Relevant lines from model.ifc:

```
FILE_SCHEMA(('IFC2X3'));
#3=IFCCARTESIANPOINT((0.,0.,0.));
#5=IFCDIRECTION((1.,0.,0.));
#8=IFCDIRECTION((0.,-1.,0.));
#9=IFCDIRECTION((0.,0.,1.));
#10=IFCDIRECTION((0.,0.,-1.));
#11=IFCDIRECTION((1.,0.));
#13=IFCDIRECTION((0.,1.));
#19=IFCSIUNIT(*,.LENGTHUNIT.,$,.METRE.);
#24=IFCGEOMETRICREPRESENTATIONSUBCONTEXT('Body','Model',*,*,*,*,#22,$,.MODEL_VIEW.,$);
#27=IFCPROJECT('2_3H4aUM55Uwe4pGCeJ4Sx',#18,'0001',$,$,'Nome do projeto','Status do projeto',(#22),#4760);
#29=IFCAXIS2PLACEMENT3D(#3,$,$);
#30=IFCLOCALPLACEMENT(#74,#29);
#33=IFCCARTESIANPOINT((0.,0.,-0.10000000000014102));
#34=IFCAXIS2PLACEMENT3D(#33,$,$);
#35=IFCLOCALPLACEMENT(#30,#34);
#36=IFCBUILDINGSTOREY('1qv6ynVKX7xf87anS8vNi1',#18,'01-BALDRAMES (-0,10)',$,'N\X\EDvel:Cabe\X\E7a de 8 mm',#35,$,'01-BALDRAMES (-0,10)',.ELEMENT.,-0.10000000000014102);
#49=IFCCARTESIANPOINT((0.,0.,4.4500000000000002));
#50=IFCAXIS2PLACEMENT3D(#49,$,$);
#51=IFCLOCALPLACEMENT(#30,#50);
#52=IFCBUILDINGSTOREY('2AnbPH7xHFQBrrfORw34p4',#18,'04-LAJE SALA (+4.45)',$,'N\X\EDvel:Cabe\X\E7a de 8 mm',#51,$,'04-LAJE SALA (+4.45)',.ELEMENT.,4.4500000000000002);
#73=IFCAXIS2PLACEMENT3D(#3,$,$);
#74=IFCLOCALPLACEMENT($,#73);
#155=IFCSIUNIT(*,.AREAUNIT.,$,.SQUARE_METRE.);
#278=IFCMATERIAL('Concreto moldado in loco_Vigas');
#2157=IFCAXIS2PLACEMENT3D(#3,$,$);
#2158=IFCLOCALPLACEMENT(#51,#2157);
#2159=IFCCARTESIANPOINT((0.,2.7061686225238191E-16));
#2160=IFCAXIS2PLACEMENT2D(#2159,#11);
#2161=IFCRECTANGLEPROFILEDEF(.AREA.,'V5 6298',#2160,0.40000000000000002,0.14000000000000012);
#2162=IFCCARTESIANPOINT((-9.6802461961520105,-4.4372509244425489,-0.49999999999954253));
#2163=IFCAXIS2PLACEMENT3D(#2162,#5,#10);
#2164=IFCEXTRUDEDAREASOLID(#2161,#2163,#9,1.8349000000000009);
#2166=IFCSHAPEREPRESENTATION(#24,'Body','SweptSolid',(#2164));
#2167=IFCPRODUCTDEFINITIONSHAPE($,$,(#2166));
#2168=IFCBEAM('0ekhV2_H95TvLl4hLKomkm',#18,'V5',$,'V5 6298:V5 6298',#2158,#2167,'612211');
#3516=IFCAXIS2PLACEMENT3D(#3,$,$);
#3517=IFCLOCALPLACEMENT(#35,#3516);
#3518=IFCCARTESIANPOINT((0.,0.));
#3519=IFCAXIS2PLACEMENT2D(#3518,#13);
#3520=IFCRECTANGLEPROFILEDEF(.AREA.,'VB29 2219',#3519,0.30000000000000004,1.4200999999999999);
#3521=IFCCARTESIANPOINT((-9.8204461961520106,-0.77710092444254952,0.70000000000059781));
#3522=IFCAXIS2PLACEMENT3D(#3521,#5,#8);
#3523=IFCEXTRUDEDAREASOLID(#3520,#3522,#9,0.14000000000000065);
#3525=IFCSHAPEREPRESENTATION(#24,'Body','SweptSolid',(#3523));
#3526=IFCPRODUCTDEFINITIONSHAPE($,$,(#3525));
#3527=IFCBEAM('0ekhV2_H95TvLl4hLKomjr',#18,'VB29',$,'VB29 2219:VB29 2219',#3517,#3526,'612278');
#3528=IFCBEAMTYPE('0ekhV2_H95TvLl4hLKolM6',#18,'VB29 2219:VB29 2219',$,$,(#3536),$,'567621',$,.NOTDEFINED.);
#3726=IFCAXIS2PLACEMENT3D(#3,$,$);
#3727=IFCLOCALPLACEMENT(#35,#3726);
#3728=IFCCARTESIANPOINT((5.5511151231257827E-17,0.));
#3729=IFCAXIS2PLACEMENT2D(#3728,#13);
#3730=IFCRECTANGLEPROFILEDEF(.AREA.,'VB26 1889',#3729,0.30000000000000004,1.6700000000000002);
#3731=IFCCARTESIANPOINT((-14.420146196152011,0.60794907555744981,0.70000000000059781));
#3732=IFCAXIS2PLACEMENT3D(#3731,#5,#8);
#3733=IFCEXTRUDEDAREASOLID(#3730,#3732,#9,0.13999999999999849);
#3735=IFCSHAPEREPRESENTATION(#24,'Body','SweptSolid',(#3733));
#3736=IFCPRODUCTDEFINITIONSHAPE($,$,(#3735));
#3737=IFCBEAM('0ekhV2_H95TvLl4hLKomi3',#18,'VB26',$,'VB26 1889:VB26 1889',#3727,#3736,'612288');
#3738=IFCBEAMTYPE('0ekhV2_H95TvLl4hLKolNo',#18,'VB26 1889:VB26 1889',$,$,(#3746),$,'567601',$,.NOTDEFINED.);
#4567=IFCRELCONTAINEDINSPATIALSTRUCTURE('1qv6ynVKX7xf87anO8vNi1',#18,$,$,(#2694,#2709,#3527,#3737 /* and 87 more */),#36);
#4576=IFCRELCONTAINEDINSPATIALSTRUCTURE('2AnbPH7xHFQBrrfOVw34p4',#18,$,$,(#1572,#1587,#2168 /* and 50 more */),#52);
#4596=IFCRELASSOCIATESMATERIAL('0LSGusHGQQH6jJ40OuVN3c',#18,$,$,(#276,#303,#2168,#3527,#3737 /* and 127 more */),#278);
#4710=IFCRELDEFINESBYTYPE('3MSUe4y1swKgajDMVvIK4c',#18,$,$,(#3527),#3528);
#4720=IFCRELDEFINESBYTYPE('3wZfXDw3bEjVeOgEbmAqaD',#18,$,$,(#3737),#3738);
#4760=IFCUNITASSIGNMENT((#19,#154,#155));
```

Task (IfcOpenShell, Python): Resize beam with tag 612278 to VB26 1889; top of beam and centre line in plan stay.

```python
import ifcopenshell
import ifcopenshell.api.type
import ifcopenshell.util.element
import ifcopenshell.util.representation

model = ifcopenshell.open("model.ifc")

member = model.by_guid("0ekhV2_H95TvLl4hLKomjr")
source = next(p for p in model.by_type("IfcRectangleProfileDef") if p.ProfileName == "VB26 1889")

body = ifcopenshell.util.representation.get_representation(member, "Model", "Body")
solid = body.Items[0]
old_profile = solid.SweptArea

# Copy the section's sizes but keep this member's own profile position.
profile = ifcopenshell.util.element.copy(model, source)
# Profiles are centred, so shift by half the change in depth to hold the top.
shift = (old_profile.XDim - profile.XDim) / 2
x, y = old_profile.Position.Location.Coordinates
up = (0.0, -1.0)  # upwards, in the solid's own plane
location = model.createIfcCartesianPoint((x + up[0] * shift, y + up[1] * shift))
profile.Position = model.createIfcAxis2Placement2D(location, old_profile.Position.RefDirection)
solid.SweptArea = profile
if not model.get_total_inverses(old_profile):
    ifcopenshell.util.element.remove_deep2(model, old_profile)

new_type = model.by_guid("0ekhV2_H95TvLl4hLKolNo")
ifcopenshell.api.type.assign_type(
    model, related_objects=[member], relating_type=new_type, should_map_representations=False
)
member.ObjectType = "VB26 1889:VB26 1889"

print(solid.SweptArea)

model.write("model_edited.ifc")
```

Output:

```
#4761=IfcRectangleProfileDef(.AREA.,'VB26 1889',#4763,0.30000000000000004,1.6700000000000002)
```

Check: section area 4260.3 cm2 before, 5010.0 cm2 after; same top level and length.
